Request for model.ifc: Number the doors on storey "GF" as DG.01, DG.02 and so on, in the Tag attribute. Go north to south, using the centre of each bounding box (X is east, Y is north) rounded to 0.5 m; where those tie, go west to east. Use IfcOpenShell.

First a look at what the model holds.

```python
import ifcopenshell
import ifcopenshell.util.element
import ifcopenshell.util.placement

model = ifcopenshell.open("model.ifc")
print(model.schema)
storey = next(s for s in model.by_type("IfcBuildingStorey") if s.Name == "GF")
doors = [e for e in ifcopenshell.util.element.get_decomposition(storey) if e.is_a("IfcDoor")]
for e in sorted(doors, key=lambda e: e.id()):
    origin = ifcopenshell.util.placement.get_local_placement(e.ObjectPlacement)[:3, 3]
    print(e.id(), e.Tag, e.Name, origin.round(2) + 0.0, sep=" | ")
```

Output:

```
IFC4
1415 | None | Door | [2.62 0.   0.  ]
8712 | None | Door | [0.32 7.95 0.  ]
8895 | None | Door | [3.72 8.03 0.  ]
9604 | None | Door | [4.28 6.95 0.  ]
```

```python
import ifcopenshell
import ifcopenshell.geom
import ifcopenshell.util.element
import ifcopenshell.util.shape

model = ifcopenshell.open("model.ifc")
settings = ifcopenshell.geom.settings()
settings.set("use-world-coords", True)


def centre(element):
    shape = ifcopenshell.geom.create_shape(settings, element)
    return ifcopenshell.util.shape.get_bbox_centroid(shape.geometry)


storey = next(s for s in model.by_type("IfcBuildingStorey") if s.Name == "GF")
doors = [e for e in ifcopenshell.util.element.get_decomposition(storey) if e.is_a("IfcDoor")]

# Insertion points can sit at a corner or the storey origin, so sort by the geometry (in metres).
centres = {e: centre(e) for e in doors}
doors.sort(key=lambda e: (-round(centres[e][1] / 0.5), centres[e][0]))

for i, e in enumerate(doors, start=1):
    number = f"DG.{i:02d}"
    e.Tag = number
    print(e.id(), number)

model.write("model_rev.ifc")
```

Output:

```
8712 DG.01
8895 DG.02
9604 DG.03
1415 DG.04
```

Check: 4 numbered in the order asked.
